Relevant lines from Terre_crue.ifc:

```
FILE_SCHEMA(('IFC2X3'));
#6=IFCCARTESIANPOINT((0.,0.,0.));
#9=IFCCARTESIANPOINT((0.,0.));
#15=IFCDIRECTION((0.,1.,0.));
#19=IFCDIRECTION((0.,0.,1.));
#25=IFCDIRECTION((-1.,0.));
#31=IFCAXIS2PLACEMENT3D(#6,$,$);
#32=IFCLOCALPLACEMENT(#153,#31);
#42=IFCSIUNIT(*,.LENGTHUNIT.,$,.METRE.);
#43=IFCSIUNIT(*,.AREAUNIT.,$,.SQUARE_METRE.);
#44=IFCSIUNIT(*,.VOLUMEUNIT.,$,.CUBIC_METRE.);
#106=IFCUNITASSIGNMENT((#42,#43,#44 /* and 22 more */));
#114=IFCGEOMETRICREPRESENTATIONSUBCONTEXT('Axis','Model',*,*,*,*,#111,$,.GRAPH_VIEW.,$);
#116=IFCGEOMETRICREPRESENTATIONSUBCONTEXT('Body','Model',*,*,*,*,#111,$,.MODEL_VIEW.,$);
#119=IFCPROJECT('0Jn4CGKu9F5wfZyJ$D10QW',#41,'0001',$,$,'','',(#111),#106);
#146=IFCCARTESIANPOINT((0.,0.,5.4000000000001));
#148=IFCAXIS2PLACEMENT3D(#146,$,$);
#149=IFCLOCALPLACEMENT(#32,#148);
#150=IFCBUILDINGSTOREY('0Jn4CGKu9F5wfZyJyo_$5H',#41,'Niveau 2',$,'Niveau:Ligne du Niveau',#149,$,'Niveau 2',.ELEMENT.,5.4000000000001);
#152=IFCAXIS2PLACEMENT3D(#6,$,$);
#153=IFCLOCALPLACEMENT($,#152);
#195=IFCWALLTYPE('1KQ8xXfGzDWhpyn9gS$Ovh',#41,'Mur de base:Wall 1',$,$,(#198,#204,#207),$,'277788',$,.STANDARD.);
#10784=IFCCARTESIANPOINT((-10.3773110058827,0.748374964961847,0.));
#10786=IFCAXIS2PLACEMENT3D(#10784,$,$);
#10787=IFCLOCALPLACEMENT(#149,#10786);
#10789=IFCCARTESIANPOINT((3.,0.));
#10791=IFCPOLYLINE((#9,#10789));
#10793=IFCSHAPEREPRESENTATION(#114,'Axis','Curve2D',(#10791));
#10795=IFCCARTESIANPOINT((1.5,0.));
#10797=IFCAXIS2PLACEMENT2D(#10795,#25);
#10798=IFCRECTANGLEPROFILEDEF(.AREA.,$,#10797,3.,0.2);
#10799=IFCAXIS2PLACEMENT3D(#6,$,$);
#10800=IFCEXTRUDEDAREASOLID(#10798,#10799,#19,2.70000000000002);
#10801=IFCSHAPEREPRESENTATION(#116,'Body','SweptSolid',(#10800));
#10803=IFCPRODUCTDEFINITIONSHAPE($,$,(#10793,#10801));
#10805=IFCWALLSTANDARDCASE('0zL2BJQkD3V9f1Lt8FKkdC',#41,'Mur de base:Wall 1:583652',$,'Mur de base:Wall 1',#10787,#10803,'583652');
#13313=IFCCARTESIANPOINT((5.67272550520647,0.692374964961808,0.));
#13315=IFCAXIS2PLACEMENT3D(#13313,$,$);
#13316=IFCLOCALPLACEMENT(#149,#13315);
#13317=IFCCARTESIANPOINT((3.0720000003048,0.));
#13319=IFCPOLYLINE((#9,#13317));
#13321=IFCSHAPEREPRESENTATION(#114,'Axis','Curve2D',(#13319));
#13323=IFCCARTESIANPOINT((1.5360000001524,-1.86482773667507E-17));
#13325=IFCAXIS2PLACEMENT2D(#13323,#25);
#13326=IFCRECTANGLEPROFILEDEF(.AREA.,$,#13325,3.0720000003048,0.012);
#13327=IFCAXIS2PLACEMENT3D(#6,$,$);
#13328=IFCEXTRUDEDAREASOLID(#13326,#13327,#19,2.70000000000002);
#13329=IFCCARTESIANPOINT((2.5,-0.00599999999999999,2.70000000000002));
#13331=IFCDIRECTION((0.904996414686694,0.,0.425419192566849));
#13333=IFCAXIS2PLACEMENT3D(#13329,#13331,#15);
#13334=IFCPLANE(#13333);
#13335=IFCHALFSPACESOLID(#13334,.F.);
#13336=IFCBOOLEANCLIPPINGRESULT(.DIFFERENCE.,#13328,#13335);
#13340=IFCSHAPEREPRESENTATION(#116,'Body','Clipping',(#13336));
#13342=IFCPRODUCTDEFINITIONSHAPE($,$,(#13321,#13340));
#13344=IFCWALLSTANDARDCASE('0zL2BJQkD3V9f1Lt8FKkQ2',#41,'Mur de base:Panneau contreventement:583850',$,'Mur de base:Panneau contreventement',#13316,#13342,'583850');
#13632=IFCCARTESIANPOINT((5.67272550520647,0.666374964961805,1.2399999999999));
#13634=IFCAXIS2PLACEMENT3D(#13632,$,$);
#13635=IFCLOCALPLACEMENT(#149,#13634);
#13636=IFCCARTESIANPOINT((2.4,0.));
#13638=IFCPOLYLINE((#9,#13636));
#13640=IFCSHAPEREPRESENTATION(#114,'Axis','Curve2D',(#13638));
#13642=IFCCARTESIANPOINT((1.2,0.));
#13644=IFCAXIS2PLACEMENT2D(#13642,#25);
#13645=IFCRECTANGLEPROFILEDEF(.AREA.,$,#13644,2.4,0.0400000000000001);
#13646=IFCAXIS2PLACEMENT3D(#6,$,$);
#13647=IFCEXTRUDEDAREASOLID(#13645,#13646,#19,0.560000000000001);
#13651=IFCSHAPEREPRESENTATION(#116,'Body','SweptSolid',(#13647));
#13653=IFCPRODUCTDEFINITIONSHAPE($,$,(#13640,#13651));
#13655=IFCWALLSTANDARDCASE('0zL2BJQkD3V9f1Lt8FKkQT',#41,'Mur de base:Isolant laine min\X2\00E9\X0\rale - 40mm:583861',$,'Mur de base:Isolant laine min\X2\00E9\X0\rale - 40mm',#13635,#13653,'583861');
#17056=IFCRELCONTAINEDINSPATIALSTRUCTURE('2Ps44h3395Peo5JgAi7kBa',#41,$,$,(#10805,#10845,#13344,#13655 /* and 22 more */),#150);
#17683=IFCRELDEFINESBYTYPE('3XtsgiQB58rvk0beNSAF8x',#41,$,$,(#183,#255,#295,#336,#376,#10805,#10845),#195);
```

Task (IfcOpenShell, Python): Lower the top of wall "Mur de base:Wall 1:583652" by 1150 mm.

```python
import ifcopenshell
import ifcopenshell.geom
import ifcopenshell.util.representation
import ifcopenshell.util.shape
import ifcopenshell.util.unit

model = ifcopenshell.open("Terre_crue.ifc")
unit_scale = ifcopenshell.util.unit.calculate_unit_scale(model)
settings = ifcopenshell.geom.settings()


def volume(element):
    """Net volume in cubic metres, openings subtracted."""
    shape = ifcopenshell.geom.create_shape(settings, element)
    return ifcopenshell.util.shape.get_volume(shape.geometry)


wall = model.by_id(10805)
before = volume(wall)

body = ifcopenshell.util.representation.get_representation(wall, "Model", "Body")
solid = body.Items[0]
old_height = solid.Depth
solid.Depth -= 1.15 / unit_scale
after = volume(wall)

print(f"height {old_height:g} -> {solid.Depth:g}, volume {before:.3f} -> {after:.3f} m3")

model.write("Terre_crue_updated.ifc")
```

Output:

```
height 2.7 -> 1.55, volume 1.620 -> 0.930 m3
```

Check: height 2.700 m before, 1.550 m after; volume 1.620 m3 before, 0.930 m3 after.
